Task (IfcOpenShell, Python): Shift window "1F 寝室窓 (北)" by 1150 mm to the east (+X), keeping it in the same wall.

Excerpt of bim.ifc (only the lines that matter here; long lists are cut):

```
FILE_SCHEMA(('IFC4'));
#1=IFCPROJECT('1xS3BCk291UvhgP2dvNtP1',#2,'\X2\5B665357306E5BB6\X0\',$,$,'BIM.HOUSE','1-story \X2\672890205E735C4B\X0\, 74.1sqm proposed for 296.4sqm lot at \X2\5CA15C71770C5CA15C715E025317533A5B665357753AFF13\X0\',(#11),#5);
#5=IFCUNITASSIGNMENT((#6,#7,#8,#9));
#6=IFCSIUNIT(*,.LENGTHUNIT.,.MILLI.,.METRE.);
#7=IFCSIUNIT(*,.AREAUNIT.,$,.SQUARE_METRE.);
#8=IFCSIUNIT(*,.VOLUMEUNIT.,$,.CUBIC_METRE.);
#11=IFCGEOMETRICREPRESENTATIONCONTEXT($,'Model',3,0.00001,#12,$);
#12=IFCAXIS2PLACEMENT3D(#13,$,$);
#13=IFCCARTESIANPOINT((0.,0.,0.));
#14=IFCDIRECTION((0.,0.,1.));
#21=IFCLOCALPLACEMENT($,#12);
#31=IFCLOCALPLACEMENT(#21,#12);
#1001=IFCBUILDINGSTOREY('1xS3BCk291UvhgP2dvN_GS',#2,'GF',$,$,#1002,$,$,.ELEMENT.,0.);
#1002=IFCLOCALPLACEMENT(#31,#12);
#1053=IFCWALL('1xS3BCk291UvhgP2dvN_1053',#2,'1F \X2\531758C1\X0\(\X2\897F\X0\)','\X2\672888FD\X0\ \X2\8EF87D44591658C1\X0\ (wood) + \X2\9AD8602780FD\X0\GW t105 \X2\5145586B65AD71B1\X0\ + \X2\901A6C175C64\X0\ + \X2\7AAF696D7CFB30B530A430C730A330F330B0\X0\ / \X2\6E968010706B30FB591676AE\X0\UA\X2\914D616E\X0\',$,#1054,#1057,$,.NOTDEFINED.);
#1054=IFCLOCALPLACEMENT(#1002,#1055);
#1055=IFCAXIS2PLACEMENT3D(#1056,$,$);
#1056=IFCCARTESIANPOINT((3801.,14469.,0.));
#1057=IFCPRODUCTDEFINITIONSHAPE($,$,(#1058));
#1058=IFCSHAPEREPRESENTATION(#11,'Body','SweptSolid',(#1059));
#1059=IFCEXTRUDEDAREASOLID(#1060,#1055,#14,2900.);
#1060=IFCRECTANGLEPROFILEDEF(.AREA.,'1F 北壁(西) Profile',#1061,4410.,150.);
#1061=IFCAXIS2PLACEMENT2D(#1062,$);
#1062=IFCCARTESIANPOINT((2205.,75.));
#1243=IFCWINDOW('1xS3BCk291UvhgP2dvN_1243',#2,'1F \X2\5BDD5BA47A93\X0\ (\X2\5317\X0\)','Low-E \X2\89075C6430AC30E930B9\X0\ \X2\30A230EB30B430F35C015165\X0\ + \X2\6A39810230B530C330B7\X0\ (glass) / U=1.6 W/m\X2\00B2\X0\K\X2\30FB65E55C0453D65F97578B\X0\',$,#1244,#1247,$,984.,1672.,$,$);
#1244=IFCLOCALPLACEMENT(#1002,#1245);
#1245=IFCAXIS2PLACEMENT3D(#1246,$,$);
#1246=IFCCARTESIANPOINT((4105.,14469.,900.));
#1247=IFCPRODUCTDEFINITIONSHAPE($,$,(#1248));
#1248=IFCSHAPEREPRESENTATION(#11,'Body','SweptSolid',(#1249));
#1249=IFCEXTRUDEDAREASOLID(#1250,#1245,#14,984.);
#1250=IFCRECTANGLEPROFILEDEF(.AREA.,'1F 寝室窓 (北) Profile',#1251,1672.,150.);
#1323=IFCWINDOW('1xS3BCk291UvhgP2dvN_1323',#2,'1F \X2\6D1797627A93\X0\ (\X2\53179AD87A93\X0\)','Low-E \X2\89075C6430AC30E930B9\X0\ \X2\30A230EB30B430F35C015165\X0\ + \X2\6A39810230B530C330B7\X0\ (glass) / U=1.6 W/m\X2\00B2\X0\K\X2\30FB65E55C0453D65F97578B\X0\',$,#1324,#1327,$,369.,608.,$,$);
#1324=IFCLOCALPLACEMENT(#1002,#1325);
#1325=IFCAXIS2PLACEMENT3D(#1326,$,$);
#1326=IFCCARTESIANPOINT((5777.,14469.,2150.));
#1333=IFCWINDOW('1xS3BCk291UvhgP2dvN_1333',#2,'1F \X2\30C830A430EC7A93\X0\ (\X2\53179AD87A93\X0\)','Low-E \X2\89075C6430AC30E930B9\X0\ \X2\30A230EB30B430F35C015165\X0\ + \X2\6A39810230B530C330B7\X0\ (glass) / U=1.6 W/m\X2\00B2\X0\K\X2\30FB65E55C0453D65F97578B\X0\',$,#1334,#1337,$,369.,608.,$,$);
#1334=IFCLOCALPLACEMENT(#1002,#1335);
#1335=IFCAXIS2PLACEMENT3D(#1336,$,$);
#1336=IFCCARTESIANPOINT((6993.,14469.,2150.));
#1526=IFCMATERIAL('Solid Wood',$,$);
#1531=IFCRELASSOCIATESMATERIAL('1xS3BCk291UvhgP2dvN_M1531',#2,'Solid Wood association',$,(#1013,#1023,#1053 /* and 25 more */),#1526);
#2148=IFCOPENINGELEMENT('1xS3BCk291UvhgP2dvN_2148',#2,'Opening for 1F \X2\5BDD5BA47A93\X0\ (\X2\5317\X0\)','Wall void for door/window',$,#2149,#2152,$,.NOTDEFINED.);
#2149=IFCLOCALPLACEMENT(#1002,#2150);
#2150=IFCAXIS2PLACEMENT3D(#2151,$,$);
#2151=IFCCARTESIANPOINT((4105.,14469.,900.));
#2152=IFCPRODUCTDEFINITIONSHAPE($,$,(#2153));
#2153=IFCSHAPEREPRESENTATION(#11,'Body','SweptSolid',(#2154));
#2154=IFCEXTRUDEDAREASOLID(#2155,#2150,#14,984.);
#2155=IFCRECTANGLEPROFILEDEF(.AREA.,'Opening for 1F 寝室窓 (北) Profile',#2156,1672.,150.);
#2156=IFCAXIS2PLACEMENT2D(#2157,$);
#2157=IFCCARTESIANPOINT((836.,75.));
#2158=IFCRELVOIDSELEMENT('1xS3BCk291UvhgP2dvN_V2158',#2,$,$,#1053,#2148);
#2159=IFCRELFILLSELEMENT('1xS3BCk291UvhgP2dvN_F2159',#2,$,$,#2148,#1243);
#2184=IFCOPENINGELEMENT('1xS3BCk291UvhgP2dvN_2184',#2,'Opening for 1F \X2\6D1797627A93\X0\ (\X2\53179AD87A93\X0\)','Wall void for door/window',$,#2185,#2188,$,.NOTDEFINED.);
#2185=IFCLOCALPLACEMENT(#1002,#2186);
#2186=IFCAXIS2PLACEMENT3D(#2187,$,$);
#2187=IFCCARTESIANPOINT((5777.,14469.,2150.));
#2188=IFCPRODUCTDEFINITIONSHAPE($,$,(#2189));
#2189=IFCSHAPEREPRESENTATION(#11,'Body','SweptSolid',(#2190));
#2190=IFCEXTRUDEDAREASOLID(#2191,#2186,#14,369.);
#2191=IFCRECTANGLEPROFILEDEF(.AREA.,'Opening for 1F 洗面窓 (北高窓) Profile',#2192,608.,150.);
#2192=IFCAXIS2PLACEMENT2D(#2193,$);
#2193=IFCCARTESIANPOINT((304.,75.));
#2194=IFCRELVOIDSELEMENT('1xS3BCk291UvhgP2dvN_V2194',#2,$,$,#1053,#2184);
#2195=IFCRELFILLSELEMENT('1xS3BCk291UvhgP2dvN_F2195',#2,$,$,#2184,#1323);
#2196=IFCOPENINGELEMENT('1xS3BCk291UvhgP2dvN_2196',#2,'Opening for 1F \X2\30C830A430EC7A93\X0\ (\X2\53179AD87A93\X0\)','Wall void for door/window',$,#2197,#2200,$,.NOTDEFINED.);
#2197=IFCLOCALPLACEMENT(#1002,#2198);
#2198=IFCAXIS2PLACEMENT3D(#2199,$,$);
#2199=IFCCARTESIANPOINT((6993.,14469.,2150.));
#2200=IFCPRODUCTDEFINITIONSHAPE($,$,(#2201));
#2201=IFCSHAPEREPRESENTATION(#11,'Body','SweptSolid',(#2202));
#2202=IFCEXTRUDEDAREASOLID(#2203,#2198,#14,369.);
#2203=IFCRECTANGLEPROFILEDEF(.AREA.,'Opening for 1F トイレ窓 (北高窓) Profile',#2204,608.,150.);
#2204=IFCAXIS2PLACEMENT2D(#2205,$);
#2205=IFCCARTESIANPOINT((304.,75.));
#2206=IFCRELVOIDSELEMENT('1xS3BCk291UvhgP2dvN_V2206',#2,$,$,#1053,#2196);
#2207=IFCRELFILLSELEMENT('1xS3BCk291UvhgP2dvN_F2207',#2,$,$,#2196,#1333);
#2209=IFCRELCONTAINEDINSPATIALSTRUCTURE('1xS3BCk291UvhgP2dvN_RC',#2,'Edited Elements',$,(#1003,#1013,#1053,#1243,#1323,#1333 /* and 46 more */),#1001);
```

```python
import ifcopenshell
import ifcopenshell.api.geometry
import ifcopenshell.util.placement

model = ifcopenshell.open("bim.ifc")

window = model.by_guid("1xS3BCk291UvhgP2dvN_1243")
opening = window.FillsVoids[0].RelatingOpeningElement
wall = opening.VoidsElements[0].RelatingBuildingElement

wall_matrix = ifcopenshell.util.placement.get_local_placement(wall.ObjectPlacement)
shift = wall_matrix[:3, 0] * 1150.0
before = ifcopenshell.util.placement.get_local_placement(window.ObjectPlacement)[:3, 3].copy()

# The window is not placed relative to its opening, so move both.
for product in (opening, window):
    matrix = ifcopenshell.util.placement.get_local_placement(product.ObjectPlacement)
    matrix[:3, 3] += shift
    ifcopenshell.api.geometry.edit_object_placement(model, product=product, matrix=matrix, is_si=False)

after = ifcopenshell.util.placement.get_local_placement(window.ObjectPlacement)[:3, 3]
print("window moved by", (after - before).round(3) + 0.0)

model.write("bim_v2.ifc")
```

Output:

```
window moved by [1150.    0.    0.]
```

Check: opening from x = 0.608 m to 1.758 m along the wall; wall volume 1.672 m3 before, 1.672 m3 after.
